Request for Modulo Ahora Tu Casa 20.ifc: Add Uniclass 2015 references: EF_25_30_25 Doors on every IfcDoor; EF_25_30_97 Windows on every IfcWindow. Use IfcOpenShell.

First a look at what the model holds.

```python
import ifcopenshell

model = ifcopenshell.open("Modulo Ahora Tu Casa 20.ifc")
print(model.schema)
print("classifications:", [c.Name for c in model.by_type("IfcClassification")])
for ifc_class in ("IfcDoor", "IfcRoof", "IfcStair", "IfcWall", "IfcWindow"):
    print(ifc_class, len(model.by_type(ifc_class)))
```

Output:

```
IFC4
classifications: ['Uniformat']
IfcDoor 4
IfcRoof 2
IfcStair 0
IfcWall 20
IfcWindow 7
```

```python
import ifcopenshell
import ifcopenshell.api.classification

model = ifcopenshell.open("Modulo Ahora Tu Casa 20.ifc")

system = ifcopenshell.api.classification.add_classification(model, classification="Uniclass 2015")

codes = {
    "IfcDoor": ("EF_25_30_25", "Doors"),
    "IfcWindow": ("EF_25_30_97", "Windows"),
}
for ifc_class, (code, name) in codes.items():
    products = model.by_type(ifc_class)
    ifcopenshell.api.classification.add_reference(
        model, products=products, classification=system, identification=code, name=name
    )
    print(code, len(products))

model.write("Modulo Ahora Tu Casa 20_edited.ifc")
```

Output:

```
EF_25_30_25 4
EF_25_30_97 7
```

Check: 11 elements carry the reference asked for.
